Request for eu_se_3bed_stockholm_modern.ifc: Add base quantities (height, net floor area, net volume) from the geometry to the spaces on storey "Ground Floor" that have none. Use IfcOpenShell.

First a look at what the model holds.

```python
import ifcopenshell
import ifcopenshell.util.element
import ifcopenshell.util.unit

model = ifcopenshell.open("eu_se_3bed_stockholm_modern.ifc")
print(model.schema)
for unit_type in ("LENGTHUNIT", "AREAUNIT", "VOLUMEUNIT"):
    print(unit_type, ifcopenshell.util.unit.calculate_unit_scale(model, unit_type))
storey = next(s for s in model.by_type("IfcBuildingStorey") if s.Name == "Ground Floor")
spaces = [e for e in ifcopenshell.util.element.get_decomposition(storey) if e.is_a("IfcSpace")]
for e in sorted(spaces, key=lambda e: e.id()):
    print(e.id(), e.is_a(), e.Name, list(ifcopenshell.util.element.get_psets(e, qtos_only=True)), sep=" | ")
```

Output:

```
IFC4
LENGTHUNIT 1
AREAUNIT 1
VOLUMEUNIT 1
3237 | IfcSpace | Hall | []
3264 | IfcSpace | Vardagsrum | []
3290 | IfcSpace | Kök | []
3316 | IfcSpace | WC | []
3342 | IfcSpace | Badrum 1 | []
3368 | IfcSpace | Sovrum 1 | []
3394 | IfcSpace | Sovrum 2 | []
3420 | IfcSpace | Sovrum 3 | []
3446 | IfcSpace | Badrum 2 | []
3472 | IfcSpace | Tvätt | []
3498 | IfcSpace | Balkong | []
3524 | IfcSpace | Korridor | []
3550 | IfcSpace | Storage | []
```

```python
import ifcopenshell
import ifcopenshell.api.pset
import ifcopenshell.geom
import ifcopenshell.util.element
import ifcopenshell.util.shape
import ifcopenshell.util.unit

model = ifcopenshell.open("eu_se_3bed_stockholm_modern.ifc")
unit_scale = ifcopenshell.util.unit.calculate_unit_scale(model)
area_scale = ifcopenshell.util.unit.calculate_unit_scale(model, "AREAUNIT")
volume_scale = ifcopenshell.util.unit.calculate_unit_scale(model, "VOLUMEUNIT")
settings = ifcopenshell.geom.settings()

storey = next(s for s in model.by_type("IfcBuildingStorey") if s.Name == "Ground Floor")
spaces = [e for e in ifcopenshell.util.element.get_decomposition(storey) if e.is_a("IfcSpace")]

for e in sorted(spaces, key=lambda e: e.id()):
    if ifcopenshell.util.element.get_psets(e, qtos_only=True, should_inherit=False):
        continue
    # Geometry comes back in metres, in the element's own axes.
    shape = ifcopenshell.geom.create_shape(settings, e)
    values = {
        "Height": ifcopenshell.util.shape.get_z(shape.geometry) / unit_scale,
        "NetFloorArea": ifcopenshell.util.shape.get_footprint_area(shape.geometry) / area_scale,
        "NetVolume": ifcopenshell.util.shape.get_volume(shape.geometry) / volume_scale,
    }
    qto = ifcopenshell.api.pset.add_qto(model, product=e, name="Qto_SpaceBaseQuantities")
    ifcopenshell.api.pset.edit_qto(model, qto=qto, properties=values)
    print(e.id(), {k: round(v, 3) for k, v in values.items()})

model.write("eu_se_3bed_stockholm_modern_edited.ifc")
```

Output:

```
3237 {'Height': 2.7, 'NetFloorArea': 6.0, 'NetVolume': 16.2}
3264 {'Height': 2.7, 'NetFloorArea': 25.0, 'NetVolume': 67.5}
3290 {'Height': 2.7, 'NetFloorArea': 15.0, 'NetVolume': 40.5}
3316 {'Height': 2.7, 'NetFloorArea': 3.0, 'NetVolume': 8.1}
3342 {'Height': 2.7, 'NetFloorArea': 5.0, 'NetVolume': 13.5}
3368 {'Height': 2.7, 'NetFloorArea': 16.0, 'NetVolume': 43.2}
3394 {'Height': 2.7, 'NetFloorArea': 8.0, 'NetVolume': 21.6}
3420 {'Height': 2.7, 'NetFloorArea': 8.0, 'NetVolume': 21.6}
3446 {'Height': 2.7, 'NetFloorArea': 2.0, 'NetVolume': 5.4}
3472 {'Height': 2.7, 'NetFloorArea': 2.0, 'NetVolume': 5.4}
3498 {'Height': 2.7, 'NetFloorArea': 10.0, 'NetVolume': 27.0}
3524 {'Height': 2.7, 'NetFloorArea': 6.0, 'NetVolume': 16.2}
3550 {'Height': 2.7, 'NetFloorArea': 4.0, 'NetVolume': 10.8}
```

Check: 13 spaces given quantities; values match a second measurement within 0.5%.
